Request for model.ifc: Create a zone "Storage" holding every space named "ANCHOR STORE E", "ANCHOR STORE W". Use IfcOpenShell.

First a look at what the model holds.

```python
import ifcopenshell

model = ifcopenshell.open("model.ifc")
print(model.schema)
seen = {}
for space in model.by_type("IfcSpace"):
    seen[space.LongName] = seen.get(space.LongName, 0) + 1
for name, count in sorted(seen.items(), key=str):
    print(count, "x", name)
print("zones:", [z.Name for z in model.by_type("IfcZone")][:20])
```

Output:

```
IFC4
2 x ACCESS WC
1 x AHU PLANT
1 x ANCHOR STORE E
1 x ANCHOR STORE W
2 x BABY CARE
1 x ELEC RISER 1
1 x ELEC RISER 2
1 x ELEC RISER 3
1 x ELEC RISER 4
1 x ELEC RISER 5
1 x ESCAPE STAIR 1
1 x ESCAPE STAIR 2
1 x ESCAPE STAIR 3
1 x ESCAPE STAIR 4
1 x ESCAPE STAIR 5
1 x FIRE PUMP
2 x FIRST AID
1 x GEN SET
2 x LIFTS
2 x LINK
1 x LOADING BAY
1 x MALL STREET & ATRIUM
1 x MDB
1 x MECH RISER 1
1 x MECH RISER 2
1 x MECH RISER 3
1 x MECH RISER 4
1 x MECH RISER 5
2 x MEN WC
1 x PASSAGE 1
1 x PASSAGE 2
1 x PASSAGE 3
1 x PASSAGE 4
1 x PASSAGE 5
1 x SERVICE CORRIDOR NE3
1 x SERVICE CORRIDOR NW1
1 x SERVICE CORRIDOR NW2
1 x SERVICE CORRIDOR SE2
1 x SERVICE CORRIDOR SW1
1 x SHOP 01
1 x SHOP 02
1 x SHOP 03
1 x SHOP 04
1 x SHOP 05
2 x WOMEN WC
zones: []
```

```python
import ifcopenshell
import ifcopenshell.api.group
import ifcopenshell.api.root

model = ifcopenshell.open("model.ifc")

names = {"ANCHOR STORE E", "ANCHOR STORE W"}
spaces = [s for s in model.by_type("IfcSpace") if s.LongName in names]

zone = ifcopenshell.api.root.create_entity(model, ifc_class="IfcZone", name="Storage")
ifcopenshell.api.group.assign_group(model, products=spaces, group=zone)
print(len(spaces), "spaces in", zone.Name)

model.write("model_rev.ifc")
```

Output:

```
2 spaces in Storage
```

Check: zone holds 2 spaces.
